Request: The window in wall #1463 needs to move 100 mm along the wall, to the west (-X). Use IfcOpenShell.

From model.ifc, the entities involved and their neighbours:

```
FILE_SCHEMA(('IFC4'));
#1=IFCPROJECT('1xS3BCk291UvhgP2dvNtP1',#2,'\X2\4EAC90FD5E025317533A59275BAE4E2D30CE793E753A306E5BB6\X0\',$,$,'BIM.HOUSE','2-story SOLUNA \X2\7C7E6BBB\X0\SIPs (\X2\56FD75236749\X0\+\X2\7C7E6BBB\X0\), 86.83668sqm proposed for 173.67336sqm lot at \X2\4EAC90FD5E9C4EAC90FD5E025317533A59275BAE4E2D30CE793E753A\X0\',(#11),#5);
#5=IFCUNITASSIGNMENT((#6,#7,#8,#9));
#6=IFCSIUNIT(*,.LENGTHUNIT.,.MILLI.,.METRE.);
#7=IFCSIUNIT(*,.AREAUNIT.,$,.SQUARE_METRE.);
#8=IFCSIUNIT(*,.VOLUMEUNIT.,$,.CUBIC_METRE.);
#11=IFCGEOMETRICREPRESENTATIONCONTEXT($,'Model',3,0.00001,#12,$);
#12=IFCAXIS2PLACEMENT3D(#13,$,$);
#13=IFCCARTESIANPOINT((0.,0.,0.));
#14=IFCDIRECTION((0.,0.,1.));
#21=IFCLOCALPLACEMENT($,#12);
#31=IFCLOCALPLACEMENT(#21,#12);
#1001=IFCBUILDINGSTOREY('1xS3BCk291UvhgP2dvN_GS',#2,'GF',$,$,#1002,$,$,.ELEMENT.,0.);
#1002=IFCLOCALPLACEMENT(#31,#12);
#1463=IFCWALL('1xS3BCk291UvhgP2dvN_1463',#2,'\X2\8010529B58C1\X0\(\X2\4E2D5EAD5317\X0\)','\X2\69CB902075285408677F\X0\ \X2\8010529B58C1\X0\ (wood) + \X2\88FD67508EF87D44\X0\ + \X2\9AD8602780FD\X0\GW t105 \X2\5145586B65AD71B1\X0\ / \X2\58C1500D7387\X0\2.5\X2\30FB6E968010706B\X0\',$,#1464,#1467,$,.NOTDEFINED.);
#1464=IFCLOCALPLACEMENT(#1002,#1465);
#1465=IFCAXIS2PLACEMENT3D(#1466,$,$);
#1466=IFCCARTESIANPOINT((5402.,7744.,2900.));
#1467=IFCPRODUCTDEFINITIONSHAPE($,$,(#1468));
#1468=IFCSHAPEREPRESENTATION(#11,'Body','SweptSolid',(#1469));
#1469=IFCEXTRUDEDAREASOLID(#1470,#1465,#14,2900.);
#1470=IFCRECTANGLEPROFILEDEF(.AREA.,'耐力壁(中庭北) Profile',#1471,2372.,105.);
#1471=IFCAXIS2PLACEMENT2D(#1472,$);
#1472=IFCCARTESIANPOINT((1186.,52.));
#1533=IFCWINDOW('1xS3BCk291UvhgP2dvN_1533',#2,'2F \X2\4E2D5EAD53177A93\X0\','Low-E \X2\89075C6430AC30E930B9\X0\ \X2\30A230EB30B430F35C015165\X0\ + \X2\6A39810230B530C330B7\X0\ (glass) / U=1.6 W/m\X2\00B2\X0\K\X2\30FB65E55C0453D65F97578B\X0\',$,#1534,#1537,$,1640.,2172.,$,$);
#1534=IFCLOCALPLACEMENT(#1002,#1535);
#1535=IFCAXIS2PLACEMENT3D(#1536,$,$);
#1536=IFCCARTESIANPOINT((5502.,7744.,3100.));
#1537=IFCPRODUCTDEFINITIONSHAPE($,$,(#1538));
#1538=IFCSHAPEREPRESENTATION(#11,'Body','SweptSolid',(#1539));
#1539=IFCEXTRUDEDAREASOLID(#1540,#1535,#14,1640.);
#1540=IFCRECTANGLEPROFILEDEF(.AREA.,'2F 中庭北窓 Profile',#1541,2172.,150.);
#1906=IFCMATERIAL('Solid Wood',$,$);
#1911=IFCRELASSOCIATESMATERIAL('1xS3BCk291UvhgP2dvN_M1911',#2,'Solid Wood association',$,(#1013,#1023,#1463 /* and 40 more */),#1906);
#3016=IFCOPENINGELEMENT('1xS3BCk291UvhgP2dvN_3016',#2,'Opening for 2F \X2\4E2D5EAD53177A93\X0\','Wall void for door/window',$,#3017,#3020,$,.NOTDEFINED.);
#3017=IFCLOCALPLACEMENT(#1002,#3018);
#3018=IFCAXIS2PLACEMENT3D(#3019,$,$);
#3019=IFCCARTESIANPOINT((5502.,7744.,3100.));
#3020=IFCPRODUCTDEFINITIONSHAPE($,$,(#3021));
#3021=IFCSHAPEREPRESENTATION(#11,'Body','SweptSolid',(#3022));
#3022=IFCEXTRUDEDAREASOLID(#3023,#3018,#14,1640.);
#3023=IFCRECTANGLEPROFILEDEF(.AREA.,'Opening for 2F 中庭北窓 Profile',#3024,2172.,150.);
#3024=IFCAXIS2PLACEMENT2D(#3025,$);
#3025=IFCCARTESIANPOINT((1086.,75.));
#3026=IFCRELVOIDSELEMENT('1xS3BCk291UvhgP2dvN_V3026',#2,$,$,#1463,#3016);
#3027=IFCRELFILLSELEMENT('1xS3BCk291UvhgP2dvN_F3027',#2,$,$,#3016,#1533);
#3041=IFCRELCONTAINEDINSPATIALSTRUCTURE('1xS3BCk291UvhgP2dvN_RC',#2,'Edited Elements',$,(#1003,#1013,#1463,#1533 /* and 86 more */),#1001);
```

```python
import ifcopenshell
import ifcopenshell.api.geometry
import ifcopenshell.util.placement
import ifcopenshell.util.unit

model = ifcopenshell.open("model.ifc")
unit_scale = ifcopenshell.util.unit.calculate_unit_scale(model)

window = model.by_id(1533)
opening = window.FillsVoids[0].RelatingOpeningElement
wall = opening.VoidsElements[0].RelatingBuildingElement

wall_matrix = ifcopenshell.util.placement.get_local_placement(wall.ObjectPlacement)
shift = wall_matrix[:3, 0] * -0.1 / unit_scale
before = ifcopenshell.util.placement.get_local_placement(window.ObjectPlacement)[:3, 3].copy()

# The window is not placed relative to its opening, so move both.
for product in (opening, window):
    matrix = ifcopenshell.util.placement.get_local_placement(product.ObjectPlacement)
    matrix[:3, 3] += shift
    ifcopenshell.api.geometry.edit_object_placement(model, product=product, matrix=matrix, is_si=False)

after = ifcopenshell.util.placement.get_local_placement(window.ObjectPlacement)[:3, 3]
print("window moved by", (after - before).round(3) + 0.0)

model.write("model_edited.ifc")
```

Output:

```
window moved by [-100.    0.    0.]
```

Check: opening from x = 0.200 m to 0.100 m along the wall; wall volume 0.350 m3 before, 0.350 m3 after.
